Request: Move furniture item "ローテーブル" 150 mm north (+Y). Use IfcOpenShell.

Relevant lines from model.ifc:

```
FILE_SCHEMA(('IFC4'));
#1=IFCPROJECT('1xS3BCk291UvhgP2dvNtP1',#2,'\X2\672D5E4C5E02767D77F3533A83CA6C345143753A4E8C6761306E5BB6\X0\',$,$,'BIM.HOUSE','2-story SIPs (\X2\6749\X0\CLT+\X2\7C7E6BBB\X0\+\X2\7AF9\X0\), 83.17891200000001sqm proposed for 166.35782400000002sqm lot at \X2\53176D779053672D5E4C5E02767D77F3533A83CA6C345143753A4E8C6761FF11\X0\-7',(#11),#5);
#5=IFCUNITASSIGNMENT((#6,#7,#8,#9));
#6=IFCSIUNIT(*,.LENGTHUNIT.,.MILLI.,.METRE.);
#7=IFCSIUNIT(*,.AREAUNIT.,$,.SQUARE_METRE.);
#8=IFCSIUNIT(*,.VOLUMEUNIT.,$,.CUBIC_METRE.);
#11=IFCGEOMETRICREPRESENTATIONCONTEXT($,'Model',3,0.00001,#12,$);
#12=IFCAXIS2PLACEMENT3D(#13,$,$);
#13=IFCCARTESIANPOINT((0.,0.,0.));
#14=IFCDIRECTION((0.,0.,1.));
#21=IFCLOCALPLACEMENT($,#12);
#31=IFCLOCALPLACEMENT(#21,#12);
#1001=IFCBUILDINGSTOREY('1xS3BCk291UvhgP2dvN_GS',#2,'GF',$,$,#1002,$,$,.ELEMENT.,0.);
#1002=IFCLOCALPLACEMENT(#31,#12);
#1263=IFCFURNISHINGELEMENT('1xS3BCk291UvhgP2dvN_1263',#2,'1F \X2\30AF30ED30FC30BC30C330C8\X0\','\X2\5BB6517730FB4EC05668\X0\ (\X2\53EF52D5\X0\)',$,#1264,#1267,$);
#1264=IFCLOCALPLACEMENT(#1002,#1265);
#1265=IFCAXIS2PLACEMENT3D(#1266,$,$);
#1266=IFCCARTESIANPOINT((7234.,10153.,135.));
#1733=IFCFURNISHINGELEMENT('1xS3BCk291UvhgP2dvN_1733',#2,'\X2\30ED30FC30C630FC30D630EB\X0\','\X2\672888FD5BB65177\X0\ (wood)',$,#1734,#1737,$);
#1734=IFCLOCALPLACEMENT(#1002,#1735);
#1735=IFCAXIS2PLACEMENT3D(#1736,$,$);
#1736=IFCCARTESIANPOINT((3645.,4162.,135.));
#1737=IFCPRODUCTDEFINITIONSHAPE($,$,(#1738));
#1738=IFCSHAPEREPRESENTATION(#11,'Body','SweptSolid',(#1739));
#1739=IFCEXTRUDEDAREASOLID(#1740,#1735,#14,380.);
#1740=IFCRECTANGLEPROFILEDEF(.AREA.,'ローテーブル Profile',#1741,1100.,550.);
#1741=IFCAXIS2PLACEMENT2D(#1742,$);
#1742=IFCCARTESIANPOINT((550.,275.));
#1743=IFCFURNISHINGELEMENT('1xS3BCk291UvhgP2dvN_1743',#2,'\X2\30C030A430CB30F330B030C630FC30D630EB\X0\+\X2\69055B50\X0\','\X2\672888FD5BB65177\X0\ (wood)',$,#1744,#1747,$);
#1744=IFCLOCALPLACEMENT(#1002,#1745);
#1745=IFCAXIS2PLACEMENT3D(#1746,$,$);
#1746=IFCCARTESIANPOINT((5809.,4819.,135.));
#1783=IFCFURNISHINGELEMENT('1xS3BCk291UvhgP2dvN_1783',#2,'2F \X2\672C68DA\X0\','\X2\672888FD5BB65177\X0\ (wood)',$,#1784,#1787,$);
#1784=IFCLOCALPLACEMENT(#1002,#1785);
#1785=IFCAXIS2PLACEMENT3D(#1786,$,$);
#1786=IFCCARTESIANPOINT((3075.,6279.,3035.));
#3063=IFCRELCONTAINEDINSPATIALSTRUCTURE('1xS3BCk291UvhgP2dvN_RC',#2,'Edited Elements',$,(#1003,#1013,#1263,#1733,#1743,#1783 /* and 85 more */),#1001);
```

```python
import ifcopenshell
import ifcopenshell.api.geometry
import ifcopenshell.util.placement
import ifcopenshell.util.unit

model = ifcopenshell.open("model.ifc")
unit_scale = ifcopenshell.util.unit.calculate_unit_scale(model)

item = model.by_guid("1xS3BCk291UvhgP2dvN_1733")
matrix = ifcopenshell.util.placement.get_local_placement(item.ObjectPlacement)
matrix[1, 3] += 0.15 / unit_scale
ifcopenshell.api.geometry.edit_object_placement(model, product=item, matrix=matrix, is_si=False)

print(ifcopenshell.util.placement.get_local_placement(item.ObjectPlacement).round(3) + 0.0)

model.write("model_rev.ifc")
```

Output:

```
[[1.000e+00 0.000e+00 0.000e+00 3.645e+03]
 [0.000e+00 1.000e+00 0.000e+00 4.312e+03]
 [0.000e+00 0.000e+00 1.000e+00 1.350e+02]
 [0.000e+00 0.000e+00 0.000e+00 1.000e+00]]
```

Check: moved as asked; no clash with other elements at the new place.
